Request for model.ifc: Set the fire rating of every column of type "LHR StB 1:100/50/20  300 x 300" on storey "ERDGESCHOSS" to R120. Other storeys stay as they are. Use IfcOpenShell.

First a look at what the model holds.

```python
import ifcopenshell
import ifcopenshell.util.element

model = ifcopenshell.open("model.ifc")
print(model.schema)
storey = next(s for s in model.by_type("IfcBuildingStorey") if s.Name == "ERDGESCHOSS")
columns = [e for e in ifcopenshell.util.element.get_decomposition(storey) if e.is_a("IfcColumn")]
seen = {}
for e in columns:
    element_type = ifcopenshell.util.element.get_type(e)
    key = (element_type.Name if element_type != e and element_type else None, ifcopenshell.util.element.get_pset(e, "Pset_ColumnCommon", "FireRating"))
    seen[key] = seen.get(key, 0) + 1
for (name, value), count in sorted(seen.items(), key=str):
    print(count, "x", name, "|", value)
```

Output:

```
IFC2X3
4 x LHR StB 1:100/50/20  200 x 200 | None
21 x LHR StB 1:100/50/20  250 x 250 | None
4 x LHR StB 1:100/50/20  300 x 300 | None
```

```python
import ifcopenshell
import ifcopenshell.api.pset
import ifcopenshell.util.element

model = ifcopenshell.open("model.ifc")

storey = next(s for s in model.by_type("IfcBuildingStorey") if s.Name == "ERDGESCHOSS")
columns = [e for e in ifcopenshell.util.element.get_decomposition(storey) if e.is_a("IfcColumn")]

count = 0
for e in columns:
    element_type = ifcopenshell.util.element.get_type(e)
    if element_type in (None, e) or element_type.Name != "LHR StB 1:100/50/20  300 x 300":
        continue
    # add_pset returns the element's existing set when there is one.
    pset = ifcopenshell.api.pset.add_pset(model, product=e, name="Pset_ColumnCommon")
    ifcopenshell.api.pset.edit_pset(model, pset=pset, properties={"FireRating": "R120"})
    count += 1

print(count, "columns updated")

model.write("model_rev.ifc")
```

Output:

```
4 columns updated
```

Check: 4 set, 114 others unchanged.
